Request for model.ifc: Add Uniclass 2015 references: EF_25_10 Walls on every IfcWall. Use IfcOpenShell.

First a look at what the model holds.

```python
import ifcopenshell

model = ifcopenshell.open("model.ifc")
print(model.schema)
print("classifications:", [c.Name for c in model.by_type("IfcClassification")])
for ifc_class in ("IfcDoor", "IfcRoof", "IfcStair", "IfcWall", "IfcWindow"):
    print(ifc_class, len(model.by_type(ifc_class)))
```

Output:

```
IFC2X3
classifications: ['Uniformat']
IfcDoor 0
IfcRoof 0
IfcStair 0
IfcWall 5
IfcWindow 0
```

```python
import ifcopenshell
import ifcopenshell.api.classification

model = ifcopenshell.open("model.ifc")

# IFC2X3 requires Source and Edition and has no link from the project to the system.
system = model.create_entity("IfcClassification", Source="NBS", Edition="2015", Name="Uniclass 2015")

codes = {
    "IfcWall": ("EF_25_10", "Walls"),
}
for ifc_class, (code, name) in codes.items():
    products = model.by_type(ifc_class)
    ifcopenshell.api.classification.add_reference(
        model, products=products, classification=system, identification=code, name=name
    )
    print(code, len(products))

model.write("model_updated.ifc")
```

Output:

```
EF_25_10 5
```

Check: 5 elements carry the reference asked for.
